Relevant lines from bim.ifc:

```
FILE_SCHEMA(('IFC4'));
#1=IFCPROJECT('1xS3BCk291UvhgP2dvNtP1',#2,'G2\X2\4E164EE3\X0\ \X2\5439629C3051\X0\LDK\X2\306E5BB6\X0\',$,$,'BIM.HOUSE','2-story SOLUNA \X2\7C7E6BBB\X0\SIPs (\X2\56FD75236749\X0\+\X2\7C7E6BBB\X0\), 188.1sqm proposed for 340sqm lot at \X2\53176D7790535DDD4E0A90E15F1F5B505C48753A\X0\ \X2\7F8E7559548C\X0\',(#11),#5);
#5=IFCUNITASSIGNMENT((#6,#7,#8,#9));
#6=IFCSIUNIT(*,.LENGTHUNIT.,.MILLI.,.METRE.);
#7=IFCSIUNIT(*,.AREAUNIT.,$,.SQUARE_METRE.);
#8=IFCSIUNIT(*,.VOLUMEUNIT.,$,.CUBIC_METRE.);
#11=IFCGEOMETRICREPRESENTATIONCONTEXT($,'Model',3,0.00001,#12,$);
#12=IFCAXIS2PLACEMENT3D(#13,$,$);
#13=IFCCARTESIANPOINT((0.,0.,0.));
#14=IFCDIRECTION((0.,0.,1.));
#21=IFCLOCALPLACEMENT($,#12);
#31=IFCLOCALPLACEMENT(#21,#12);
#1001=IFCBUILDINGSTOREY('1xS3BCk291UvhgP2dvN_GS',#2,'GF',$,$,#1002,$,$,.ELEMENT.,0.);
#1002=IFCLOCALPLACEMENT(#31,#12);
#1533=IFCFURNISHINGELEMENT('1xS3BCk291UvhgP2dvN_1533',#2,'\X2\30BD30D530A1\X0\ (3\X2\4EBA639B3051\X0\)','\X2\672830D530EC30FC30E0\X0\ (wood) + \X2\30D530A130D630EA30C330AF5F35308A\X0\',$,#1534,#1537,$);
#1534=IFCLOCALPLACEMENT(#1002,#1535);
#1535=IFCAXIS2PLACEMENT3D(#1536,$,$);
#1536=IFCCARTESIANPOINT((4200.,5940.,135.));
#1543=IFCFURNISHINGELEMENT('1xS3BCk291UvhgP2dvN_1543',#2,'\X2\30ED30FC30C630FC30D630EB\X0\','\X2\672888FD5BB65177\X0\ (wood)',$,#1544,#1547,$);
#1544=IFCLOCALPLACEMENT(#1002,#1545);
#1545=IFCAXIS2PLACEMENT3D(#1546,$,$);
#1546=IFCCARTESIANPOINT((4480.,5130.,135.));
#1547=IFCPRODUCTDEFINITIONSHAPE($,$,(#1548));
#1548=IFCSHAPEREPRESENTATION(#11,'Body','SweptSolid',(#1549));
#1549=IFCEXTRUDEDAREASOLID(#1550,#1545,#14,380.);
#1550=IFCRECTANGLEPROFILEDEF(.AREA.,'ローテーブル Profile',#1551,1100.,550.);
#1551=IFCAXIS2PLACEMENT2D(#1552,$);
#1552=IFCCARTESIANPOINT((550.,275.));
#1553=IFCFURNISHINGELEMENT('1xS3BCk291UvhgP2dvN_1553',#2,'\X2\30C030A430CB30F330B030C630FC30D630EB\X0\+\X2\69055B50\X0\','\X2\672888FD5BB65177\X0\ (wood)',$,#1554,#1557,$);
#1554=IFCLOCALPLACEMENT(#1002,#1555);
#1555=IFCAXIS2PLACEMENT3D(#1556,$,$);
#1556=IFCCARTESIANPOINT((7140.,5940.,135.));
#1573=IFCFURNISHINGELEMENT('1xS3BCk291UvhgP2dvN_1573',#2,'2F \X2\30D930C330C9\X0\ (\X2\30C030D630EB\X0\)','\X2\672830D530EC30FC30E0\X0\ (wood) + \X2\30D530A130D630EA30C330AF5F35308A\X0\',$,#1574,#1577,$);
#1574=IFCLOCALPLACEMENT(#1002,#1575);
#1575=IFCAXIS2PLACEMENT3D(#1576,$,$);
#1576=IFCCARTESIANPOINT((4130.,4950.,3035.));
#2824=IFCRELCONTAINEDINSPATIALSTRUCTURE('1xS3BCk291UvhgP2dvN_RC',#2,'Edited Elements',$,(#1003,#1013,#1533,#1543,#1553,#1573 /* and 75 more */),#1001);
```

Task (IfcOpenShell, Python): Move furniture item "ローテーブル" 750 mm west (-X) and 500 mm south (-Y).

```python
import ifcopenshell
import ifcopenshell.api.geometry
import ifcopenshell.util.placement
import ifcopenshell.util.unit

model = ifcopenshell.open("bim.ifc")
unit_scale = ifcopenshell.util.unit.calculate_unit_scale(model)

item = model.by_id(1543)
matrix = ifcopenshell.util.placement.get_local_placement(item.ObjectPlacement)
matrix[0, 3] -= 0.75 / unit_scale
matrix[1, 3] -= 0.5 / unit_scale
ifcopenshell.api.geometry.edit_object_placement(model, product=item, matrix=matrix, is_si=False)

print(ifcopenshell.util.placement.get_local_placement(item.ObjectPlacement).round(3) + 0.0)

model.write("bim-out.ifc")
```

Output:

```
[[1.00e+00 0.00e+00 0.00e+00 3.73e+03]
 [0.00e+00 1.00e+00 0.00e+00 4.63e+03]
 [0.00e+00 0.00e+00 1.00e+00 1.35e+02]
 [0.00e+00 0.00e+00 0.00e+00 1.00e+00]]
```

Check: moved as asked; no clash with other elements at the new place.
